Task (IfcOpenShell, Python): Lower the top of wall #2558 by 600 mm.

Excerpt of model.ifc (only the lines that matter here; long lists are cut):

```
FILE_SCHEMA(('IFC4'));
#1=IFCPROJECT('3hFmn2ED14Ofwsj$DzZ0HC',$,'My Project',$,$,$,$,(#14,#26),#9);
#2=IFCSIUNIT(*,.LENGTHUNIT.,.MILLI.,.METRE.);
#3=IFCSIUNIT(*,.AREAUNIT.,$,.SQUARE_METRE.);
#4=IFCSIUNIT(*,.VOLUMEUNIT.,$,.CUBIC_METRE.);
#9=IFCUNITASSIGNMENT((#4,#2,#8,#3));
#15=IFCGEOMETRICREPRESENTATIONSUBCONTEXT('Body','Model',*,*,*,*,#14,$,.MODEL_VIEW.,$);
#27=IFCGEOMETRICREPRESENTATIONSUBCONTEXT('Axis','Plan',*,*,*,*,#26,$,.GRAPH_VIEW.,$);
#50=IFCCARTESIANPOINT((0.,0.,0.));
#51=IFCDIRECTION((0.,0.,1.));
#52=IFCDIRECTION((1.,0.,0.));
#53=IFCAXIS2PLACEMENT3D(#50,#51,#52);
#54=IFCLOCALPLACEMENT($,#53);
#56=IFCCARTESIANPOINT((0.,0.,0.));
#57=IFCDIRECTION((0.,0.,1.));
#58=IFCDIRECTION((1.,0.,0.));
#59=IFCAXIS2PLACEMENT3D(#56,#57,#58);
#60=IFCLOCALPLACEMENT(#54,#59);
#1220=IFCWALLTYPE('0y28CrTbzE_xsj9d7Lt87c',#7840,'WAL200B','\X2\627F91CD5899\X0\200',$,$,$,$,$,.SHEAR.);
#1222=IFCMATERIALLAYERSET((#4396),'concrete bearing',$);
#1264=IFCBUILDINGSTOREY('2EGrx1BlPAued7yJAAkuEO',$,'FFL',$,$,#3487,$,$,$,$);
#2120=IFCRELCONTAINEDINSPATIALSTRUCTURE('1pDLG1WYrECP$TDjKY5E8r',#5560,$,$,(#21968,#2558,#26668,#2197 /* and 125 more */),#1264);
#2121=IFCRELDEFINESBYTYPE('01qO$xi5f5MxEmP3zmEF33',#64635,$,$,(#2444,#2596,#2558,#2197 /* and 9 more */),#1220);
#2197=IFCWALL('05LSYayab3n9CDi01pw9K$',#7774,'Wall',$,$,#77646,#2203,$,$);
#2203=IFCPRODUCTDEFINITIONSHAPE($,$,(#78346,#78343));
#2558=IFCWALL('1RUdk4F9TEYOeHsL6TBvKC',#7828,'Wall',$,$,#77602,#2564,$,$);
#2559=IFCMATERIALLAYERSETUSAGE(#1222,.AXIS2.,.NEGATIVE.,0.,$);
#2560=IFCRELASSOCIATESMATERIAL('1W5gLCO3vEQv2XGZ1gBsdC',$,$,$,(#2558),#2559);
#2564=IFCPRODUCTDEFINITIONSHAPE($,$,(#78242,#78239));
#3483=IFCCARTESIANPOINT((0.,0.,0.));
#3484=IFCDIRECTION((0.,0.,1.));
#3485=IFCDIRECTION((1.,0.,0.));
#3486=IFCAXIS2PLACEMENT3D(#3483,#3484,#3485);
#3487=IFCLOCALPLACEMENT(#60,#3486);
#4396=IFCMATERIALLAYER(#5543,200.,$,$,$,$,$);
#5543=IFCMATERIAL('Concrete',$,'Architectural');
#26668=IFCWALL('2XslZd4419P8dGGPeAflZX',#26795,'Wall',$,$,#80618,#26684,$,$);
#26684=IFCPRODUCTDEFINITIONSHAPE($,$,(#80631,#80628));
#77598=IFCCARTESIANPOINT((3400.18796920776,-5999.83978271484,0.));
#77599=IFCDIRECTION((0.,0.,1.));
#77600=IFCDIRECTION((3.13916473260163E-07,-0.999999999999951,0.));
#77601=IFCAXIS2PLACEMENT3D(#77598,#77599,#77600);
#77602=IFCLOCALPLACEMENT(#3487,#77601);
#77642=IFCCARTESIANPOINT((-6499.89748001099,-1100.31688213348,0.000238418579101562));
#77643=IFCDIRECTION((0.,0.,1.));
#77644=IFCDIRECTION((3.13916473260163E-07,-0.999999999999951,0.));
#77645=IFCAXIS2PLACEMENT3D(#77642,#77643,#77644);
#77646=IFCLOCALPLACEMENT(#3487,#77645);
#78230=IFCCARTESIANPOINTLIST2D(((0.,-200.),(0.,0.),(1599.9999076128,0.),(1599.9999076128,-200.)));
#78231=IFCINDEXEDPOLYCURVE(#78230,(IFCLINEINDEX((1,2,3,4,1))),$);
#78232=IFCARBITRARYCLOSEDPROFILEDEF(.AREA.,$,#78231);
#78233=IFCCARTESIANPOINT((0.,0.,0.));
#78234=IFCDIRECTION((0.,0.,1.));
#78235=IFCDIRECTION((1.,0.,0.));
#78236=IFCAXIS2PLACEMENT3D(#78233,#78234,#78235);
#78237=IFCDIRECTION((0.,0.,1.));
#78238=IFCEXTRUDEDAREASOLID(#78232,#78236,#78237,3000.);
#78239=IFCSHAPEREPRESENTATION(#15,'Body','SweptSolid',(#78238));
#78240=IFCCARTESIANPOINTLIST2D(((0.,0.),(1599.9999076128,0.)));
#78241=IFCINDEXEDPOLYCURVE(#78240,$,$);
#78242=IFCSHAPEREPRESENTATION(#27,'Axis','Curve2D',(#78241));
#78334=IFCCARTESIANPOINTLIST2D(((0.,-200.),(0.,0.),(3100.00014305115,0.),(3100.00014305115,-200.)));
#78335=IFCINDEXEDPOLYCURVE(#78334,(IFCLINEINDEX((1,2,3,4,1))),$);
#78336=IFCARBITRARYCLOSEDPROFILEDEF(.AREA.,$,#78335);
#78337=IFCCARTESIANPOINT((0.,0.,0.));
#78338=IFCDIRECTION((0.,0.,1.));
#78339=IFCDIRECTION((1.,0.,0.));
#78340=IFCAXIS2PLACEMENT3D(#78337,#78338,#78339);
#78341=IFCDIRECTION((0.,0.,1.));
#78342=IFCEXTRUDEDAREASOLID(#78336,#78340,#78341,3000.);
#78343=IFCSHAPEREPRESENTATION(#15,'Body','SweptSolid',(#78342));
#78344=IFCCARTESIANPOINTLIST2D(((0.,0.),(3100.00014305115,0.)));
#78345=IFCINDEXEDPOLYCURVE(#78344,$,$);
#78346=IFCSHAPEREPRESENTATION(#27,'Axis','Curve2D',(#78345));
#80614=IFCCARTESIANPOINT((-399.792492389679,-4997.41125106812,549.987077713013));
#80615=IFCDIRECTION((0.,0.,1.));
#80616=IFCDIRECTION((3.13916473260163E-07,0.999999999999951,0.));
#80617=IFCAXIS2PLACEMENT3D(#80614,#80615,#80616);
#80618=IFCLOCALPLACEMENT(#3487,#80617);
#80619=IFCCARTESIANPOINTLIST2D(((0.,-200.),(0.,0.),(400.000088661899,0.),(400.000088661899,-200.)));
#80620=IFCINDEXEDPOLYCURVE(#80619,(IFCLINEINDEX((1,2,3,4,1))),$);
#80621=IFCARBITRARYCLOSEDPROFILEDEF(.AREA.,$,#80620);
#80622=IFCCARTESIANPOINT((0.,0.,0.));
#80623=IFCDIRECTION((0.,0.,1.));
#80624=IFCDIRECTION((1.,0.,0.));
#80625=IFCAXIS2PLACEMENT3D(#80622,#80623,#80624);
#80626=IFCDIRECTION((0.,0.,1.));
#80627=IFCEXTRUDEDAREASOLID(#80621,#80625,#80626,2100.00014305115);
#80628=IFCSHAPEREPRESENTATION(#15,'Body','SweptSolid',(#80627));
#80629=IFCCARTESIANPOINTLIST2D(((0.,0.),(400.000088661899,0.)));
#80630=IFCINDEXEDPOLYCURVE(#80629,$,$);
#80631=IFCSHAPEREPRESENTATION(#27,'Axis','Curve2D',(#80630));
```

```python
import ifcopenshell
import ifcopenshell.geom
import ifcopenshell.util.representation
import ifcopenshell.util.shape
import ifcopenshell.util.unit

model = ifcopenshell.open("model.ifc")
unit_scale = ifcopenshell.util.unit.calculate_unit_scale(model)
settings = ifcopenshell.geom.settings()


def volume(element):
    """Net volume in cubic metres, openings subtracted."""
    shape = ifcopenshell.geom.create_shape(settings, element)
    return ifcopenshell.util.shape.get_volume(shape.geometry)


wall = model.by_id(2558)
before = volume(wall)

body = ifcopenshell.util.representation.get_representation(wall, "Model", "Body")
solid = body.Items[0]
old_height = solid.Depth
solid.Depth -= 0.6 / unit_scale
after = volume(wall)

print(f"height {old_height:g} -> {solid.Depth:g}, volume {before:.3f} -> {after:.3f} m3")

model.write("model_edited.ifc")
```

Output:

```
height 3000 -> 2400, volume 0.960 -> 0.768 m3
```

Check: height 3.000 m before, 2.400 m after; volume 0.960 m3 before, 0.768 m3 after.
